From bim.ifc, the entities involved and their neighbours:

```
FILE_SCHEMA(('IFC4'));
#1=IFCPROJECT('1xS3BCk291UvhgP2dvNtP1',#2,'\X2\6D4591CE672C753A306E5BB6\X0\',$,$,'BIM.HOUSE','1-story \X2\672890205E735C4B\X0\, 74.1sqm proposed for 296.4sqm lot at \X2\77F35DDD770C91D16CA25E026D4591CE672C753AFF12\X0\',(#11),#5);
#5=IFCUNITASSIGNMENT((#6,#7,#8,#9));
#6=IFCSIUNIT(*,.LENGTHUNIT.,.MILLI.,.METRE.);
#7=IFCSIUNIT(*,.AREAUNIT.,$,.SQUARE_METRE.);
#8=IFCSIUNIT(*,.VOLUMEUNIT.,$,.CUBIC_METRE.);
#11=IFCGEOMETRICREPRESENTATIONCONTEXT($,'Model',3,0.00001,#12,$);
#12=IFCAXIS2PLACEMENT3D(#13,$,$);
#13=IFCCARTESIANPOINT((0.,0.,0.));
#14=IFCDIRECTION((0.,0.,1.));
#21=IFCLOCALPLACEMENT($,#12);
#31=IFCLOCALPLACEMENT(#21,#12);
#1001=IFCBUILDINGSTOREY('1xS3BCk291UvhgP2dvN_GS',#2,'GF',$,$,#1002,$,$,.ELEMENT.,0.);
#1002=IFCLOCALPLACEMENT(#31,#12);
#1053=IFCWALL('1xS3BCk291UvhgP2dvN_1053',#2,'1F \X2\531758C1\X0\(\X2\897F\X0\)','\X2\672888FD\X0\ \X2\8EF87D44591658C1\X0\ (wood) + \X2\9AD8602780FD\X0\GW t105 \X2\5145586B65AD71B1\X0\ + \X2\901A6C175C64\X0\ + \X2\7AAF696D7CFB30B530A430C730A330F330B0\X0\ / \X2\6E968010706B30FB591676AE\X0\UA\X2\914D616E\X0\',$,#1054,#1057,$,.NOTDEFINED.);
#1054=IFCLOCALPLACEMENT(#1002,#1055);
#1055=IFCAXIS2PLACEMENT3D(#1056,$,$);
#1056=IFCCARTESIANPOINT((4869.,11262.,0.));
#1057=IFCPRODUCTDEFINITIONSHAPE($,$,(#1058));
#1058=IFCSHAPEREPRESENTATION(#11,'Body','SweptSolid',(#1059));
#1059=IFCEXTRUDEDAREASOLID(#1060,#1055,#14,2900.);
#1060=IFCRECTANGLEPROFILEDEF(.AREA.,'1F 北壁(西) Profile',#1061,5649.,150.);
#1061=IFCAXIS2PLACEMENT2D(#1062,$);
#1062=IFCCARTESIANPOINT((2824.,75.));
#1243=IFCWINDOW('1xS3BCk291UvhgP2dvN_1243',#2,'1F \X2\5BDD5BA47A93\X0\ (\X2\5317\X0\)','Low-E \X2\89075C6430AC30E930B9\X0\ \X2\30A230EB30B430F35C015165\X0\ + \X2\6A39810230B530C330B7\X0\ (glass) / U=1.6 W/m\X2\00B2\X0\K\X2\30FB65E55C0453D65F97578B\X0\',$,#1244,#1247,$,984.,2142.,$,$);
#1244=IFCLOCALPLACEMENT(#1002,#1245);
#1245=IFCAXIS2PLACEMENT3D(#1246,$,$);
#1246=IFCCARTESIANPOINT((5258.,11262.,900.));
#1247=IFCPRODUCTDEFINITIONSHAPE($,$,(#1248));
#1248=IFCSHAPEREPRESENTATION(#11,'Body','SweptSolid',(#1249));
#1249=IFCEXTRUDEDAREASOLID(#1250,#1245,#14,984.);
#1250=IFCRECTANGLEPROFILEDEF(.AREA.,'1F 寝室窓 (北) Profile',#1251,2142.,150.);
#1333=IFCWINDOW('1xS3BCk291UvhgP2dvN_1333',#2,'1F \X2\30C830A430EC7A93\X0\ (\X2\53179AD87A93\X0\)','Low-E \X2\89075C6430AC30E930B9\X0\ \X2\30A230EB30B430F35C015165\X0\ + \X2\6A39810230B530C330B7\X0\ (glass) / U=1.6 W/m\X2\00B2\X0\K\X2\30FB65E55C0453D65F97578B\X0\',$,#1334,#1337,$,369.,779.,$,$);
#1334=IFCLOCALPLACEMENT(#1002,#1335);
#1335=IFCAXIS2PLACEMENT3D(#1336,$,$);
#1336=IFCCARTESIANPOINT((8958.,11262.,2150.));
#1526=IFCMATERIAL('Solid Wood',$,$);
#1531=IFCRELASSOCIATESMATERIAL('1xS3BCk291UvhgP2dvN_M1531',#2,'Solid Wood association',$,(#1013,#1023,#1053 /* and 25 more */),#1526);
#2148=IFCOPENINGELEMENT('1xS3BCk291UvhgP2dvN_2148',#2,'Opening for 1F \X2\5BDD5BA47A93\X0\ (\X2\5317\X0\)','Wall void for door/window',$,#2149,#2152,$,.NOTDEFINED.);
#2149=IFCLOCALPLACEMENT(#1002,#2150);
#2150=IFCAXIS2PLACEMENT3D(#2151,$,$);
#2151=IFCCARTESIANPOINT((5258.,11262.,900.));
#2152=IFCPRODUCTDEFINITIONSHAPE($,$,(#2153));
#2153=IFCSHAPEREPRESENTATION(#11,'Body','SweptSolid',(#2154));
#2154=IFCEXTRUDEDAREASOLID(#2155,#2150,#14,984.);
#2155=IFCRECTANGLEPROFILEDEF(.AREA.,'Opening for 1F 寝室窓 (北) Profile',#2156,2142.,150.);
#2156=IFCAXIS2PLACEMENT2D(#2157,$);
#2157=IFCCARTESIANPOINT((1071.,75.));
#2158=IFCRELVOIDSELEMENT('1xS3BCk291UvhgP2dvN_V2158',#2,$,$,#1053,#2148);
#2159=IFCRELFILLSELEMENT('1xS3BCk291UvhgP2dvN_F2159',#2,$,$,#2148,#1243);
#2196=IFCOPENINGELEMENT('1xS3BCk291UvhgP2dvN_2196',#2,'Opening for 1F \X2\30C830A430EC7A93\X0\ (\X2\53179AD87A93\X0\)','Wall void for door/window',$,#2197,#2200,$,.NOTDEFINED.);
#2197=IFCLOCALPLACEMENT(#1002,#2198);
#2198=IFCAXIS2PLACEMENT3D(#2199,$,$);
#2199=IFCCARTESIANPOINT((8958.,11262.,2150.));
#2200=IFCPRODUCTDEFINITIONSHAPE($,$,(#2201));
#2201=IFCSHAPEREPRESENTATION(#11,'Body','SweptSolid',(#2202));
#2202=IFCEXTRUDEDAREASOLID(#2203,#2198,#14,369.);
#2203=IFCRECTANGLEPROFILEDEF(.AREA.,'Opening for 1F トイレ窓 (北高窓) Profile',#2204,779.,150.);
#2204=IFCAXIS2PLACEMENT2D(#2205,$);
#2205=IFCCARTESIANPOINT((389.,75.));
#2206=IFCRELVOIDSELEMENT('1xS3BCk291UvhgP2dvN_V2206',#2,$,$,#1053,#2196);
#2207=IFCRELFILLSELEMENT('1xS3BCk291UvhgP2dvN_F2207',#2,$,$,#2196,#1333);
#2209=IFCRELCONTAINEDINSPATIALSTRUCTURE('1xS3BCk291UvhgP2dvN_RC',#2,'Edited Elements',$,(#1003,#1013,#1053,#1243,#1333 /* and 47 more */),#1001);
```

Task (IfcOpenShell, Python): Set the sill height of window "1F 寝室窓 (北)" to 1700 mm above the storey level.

```python
import numpy as np
import ifcopenshell
import ifcopenshell.api.geometry
import ifcopenshell.geom
import ifcopenshell.util.element
import ifcopenshell.util.placement
import ifcopenshell.util.shape
import ifcopenshell.util.unit

model = ifcopenshell.open("bim.ifc")
unit_scale = ifcopenshell.util.unit.calculate_unit_scale(model)

window = model.by_guid("1xS3BCk291UvhgP2dvN_1243")
opening = window.FillsVoids[0].RelatingOpeningElement
storey = ifcopenshell.util.element.get_container(window, ifc_class="IfcBuildingStorey")
level = ifcopenshell.util.placement.get_local_placement(storey.ObjectPlacement)[2, 3]

# The opening's origin need not be at the sill, so measure its lowest point.
shape = ifcopenshell.geom.create_shape(ifcopenshell.geom.settings(), opening)
bottom = ifcopenshell.util.shape.get_shape_bottom_elevation(shape, shape.geometry) / unit_scale
dz = level + 1700.0 - bottom

shift = np.array([0.0, 0.0, dz])
# The window is not placed relative to its opening, so move both.
for product in (opening, window):
    matrix = ifcopenshell.util.placement.get_local_placement(product.ObjectPlacement)
    matrix[:3, 3] += shift
    ifcopenshell.api.geometry.edit_object_placement(model, product=product, matrix=matrix, is_si=False)

print(f"moved by {dz * unit_scale:+.3f} m")

model.write("bim_updated.ifc")
```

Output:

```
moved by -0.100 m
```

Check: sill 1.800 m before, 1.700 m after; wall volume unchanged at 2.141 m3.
